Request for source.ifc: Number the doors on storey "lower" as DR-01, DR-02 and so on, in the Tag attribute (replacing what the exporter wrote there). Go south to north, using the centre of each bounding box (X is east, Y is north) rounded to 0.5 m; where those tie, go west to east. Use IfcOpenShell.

First a look at what the model holds.

```python
import ifcopenshell
import ifcopenshell.util.element
import ifcopenshell.util.placement

model = ifcopenshell.open("source.ifc")
print(model.schema)
storey = next(s for s in model.by_type("IfcBuildingStorey") if s.Name == "lower")
doors = [e for e in ifcopenshell.util.element.get_decomposition(storey) if e.is_a("IfcDoor")]
for e in sorted(doors, key=lambda e: e.id()):
    origin = ifcopenshell.util.placement.get_local_placement(e.ObjectPlacement)[:3, 3]
    print(e.id(), e.Tag, e.Name, origin.round(2) + 0.0, sep=" | ")
```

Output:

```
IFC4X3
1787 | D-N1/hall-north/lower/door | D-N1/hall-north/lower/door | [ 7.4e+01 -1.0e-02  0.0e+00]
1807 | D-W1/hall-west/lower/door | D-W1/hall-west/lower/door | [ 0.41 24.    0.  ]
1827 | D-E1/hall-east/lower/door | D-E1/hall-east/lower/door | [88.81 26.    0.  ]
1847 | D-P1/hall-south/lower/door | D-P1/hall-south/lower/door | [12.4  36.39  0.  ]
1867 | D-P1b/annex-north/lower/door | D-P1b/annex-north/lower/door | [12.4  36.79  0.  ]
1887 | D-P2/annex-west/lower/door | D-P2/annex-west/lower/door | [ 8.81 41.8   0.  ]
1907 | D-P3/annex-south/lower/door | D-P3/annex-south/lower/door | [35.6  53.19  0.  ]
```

```python
import ifcopenshell
import ifcopenshell.geom
import ifcopenshell.util.element
import ifcopenshell.util.shape

model = ifcopenshell.open("source.ifc")
settings = ifcopenshell.geom.settings()
settings.set("use-world-coords", True)


def centre(element):
    shape = ifcopenshell.geom.create_shape(settings, element)
    return ifcopenshell.util.shape.get_bbox_centroid(shape.geometry)


storey = next(s for s in model.by_type("IfcBuildingStorey") if s.Name == "lower")
doors = [e for e in ifcopenshell.util.element.get_decomposition(storey) if e.is_a("IfcDoor")]

# Insertion points can sit at a corner or the storey origin, so sort by the geometry (in metres).
centres = {e: centre(e) for e in doors}
doors.sort(key=lambda e: (round(centres[e][1] / 0.5), centres[e][0]))

for i, e in enumerate(doors, start=1):
    number = f"DR-{i:02d}"
    e.Tag = number
    print(e.id(), number)

model.write("source_updated.ifc")
```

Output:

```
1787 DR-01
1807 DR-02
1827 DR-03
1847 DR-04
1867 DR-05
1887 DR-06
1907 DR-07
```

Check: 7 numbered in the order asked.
